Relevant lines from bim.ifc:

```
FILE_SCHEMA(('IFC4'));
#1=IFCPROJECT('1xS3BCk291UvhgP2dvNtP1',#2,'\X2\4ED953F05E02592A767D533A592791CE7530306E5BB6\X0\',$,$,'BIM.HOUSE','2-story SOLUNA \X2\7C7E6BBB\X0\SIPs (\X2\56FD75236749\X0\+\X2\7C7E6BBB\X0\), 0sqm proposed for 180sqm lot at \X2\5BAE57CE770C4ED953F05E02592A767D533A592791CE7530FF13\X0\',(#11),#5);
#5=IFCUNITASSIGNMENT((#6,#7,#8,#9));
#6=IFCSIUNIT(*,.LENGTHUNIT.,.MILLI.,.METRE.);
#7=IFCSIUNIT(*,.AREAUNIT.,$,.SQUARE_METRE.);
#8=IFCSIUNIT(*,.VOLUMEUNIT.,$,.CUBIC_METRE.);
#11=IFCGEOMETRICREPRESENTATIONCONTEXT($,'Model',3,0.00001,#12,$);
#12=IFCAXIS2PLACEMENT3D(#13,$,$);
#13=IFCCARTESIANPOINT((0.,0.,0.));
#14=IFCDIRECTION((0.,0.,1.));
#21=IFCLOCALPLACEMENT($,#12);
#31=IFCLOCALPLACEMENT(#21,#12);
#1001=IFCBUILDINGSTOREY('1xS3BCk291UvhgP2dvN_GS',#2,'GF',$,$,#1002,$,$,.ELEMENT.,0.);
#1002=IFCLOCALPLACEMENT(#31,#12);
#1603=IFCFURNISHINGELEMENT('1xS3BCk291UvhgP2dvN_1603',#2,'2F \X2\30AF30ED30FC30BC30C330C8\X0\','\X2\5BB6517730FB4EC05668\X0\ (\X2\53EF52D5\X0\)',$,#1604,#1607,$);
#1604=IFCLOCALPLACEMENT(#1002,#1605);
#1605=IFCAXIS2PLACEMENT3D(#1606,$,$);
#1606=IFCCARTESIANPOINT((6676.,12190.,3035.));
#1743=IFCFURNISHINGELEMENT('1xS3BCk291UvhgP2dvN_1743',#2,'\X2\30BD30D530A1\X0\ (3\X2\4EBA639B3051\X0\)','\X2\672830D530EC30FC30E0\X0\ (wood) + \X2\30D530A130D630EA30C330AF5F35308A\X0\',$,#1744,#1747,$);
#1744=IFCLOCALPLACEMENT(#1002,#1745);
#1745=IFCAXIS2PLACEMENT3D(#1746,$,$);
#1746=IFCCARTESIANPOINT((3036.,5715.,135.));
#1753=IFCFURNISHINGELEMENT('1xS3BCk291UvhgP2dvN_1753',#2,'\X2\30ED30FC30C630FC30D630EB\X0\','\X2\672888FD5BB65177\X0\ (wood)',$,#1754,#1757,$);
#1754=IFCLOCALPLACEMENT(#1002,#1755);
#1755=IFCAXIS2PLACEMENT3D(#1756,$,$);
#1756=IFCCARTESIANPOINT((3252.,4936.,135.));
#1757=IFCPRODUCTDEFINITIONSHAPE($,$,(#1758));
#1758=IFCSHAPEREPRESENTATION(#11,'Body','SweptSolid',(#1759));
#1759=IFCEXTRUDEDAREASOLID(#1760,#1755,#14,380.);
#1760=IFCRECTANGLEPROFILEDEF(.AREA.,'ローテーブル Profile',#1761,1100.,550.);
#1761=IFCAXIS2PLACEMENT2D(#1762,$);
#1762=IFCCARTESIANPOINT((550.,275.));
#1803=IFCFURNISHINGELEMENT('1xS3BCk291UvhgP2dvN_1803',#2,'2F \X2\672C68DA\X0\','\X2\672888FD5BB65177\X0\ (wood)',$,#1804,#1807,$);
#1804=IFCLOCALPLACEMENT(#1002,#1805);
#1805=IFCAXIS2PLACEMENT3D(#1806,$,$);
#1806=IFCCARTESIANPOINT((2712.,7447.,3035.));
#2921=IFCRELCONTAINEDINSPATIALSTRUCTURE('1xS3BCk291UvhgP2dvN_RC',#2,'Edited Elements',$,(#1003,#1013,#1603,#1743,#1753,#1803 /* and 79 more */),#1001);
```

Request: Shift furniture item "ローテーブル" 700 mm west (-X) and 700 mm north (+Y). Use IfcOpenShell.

```python
import ifcopenshell
import ifcopenshell.api.geometry
import ifcopenshell.util.placement

model = ifcopenshell.open("bim.ifc")

item = model.by_id(1753)
matrix = ifcopenshell.util.placement.get_local_placement(item.ObjectPlacement)
matrix[0, 3] -= 700.0
matrix[1, 3] += 700.0
ifcopenshell.api.geometry.edit_object_placement(model, product=item, matrix=matrix, is_si=False)

print(ifcopenshell.util.placement.get_local_placement(item.ObjectPlacement).round(3) + 0.0)

model.write("bim_edited.ifc")
```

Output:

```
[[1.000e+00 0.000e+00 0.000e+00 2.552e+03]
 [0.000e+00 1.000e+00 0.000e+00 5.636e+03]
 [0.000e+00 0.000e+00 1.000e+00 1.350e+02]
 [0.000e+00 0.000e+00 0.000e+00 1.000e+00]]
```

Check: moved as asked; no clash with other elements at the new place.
